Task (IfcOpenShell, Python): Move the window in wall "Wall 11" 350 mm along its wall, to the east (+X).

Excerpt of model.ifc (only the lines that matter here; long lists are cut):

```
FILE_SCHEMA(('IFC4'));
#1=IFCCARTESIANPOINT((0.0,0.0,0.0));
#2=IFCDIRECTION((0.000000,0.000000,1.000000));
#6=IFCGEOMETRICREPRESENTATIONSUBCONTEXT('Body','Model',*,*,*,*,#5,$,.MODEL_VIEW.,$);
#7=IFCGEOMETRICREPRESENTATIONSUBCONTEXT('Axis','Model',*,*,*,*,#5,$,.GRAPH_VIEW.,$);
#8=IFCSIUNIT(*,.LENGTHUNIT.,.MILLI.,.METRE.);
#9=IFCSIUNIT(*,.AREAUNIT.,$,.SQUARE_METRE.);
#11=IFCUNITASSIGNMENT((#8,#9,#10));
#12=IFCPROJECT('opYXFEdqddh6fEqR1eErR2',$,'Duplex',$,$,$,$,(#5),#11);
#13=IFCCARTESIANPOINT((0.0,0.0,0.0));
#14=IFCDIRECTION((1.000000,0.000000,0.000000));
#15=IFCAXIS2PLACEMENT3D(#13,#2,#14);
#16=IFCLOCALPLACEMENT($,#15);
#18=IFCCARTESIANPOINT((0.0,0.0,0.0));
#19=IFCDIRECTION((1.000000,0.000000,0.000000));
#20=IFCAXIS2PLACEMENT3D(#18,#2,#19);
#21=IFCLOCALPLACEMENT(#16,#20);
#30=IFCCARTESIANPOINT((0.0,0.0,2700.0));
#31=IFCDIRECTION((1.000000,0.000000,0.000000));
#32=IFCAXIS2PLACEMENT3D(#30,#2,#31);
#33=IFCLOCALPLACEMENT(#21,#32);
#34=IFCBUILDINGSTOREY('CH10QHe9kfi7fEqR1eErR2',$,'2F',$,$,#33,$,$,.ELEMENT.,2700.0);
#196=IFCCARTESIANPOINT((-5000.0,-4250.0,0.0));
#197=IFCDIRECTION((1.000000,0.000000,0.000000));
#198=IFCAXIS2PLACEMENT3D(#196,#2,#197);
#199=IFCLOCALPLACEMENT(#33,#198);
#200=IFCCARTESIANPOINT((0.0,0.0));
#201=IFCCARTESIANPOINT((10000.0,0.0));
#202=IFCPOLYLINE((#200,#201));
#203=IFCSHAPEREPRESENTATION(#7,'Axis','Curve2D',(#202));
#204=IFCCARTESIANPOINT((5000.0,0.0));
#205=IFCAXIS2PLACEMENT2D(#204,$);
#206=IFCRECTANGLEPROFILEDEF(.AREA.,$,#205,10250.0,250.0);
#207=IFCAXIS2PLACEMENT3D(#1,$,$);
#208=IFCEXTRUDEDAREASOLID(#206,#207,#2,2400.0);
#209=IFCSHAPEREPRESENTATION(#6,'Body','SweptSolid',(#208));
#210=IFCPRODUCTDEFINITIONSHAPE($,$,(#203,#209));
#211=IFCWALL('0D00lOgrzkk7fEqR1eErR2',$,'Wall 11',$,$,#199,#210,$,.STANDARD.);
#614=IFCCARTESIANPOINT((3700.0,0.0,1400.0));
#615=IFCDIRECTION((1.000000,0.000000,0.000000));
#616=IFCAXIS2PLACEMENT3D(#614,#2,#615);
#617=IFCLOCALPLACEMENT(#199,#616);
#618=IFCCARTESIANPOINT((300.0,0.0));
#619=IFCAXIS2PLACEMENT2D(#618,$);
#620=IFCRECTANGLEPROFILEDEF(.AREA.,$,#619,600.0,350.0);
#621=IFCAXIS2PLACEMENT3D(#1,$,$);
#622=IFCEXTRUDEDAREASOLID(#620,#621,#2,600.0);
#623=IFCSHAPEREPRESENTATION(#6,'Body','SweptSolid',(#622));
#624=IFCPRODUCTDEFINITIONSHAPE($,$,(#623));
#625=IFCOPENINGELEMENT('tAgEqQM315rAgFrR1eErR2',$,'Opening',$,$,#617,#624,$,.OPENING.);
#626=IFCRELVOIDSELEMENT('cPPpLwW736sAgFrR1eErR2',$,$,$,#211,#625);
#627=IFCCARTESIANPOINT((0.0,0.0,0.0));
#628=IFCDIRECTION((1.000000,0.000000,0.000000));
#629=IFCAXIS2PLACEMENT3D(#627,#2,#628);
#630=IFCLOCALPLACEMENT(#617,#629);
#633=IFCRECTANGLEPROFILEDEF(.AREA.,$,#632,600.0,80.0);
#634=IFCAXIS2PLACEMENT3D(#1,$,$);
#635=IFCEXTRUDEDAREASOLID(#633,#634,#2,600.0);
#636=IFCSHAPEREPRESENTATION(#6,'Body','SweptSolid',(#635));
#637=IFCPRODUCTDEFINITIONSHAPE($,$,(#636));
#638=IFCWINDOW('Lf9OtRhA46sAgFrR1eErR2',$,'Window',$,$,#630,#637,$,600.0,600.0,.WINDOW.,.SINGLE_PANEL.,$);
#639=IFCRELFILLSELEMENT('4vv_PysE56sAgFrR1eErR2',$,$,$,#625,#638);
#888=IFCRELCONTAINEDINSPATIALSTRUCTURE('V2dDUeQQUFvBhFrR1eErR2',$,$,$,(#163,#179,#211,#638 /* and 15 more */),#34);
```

```python
import ifcopenshell
import ifcopenshell.api.geometry
import ifcopenshell.util.placement
import ifcopenshell.util.unit

model = ifcopenshell.open("model.ifc")
unit_scale = ifcopenshell.util.unit.calculate_unit_scale(model)

window = model.by_guid("Lf9OtRhA46sAgFrR1eErR2")
opening = window.FillsVoids[0].RelatingOpeningElement
wall = opening.VoidsElements[0].RelatingBuildingElement

wall_matrix = ifcopenshell.util.placement.get_local_placement(wall.ObjectPlacement)
shift = wall_matrix[:3, 0] * 0.35 / unit_scale
before = ifcopenshell.util.placement.get_local_placement(window.ObjectPlacement)[:3, 3].copy()

# The window is placed relative to its opening, so it follows when the opening moves.
matrix = ifcopenshell.util.placement.get_local_placement(opening.ObjectPlacement)
matrix[:3, 3] += shift
ifcopenshell.api.geometry.edit_object_placement(
    model, product=opening, matrix=matrix, is_si=False, should_transform_children=True
)

after = ifcopenshell.util.placement.get_local_placement(window.ObjectPlacement)[:3, 3]
print("window moved by", (after - before).round(3) + 0.0)

model.write("model_rev.ifc")
```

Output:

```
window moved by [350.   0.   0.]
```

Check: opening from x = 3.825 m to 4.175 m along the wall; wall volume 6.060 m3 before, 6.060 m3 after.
